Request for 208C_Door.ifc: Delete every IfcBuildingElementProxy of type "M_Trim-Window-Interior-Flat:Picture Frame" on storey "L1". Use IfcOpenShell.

First a look at what the model holds.

```python
import ifcopenshell
import ifcopenshell.util.element

model = ifcopenshell.open("208C_Door.ifc")
print(model.schema)
storey = next(s for s in model.by_type("IfcBuildingStorey") if s.Name == "L1")
proxies = [e for e in ifcopenshell.util.element.get_decomposition(storey) if e.is_a("IfcBuildingElementProxy")]
seen = {}
for e in proxies:
    element_type = ifcopenshell.util.element.get_type(e)
    name = element_type.Name if element_type not in (None, e) else None
    seen[name] = seen.get(name, 0) + 1
for name, count in sorted(seen.items(), key=str):
    print(count, "x", name)
```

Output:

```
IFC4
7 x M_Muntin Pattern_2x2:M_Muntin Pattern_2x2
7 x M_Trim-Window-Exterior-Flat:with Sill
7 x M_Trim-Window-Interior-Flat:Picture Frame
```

```python
import ifcopenshell
import ifcopenshell.api.root
import ifcopenshell.util.element

model = ifcopenshell.open("208C_Door.ifc")

storey = next(s for s in model.by_type("IfcBuildingStorey") if s.Name == "L1")
proxies = [e for e in ifcopenshell.util.element.get_decomposition(storey) if e.is_a("IfcBuildingElementProxy")]
targets = [e for e in proxies if (t := ifcopenshell.util.element.get_type(e)) not in (None, e) and t.Name == "M_Trim-Window-Interior-Flat:Picture Frame"]

for e in targets:
    ifcopenshell.api.root.remove_product(model, product=e)
print(len(targets), "removed")

model.write("208C_Door_edited.ifc")
```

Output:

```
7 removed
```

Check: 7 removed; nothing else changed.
